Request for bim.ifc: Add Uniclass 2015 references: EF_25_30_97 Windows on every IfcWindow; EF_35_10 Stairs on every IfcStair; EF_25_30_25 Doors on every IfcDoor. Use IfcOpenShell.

First a look at what the model holds.

```python
import ifcopenshell

model = ifcopenshell.open("bim.ifc")
print(model.schema)
print("classifications:", [c.Name for c in model.by_type("IfcClassification")])
for ifc_class in ("IfcDoor", "IfcRoof", "IfcStair", "IfcWall", "IfcWindow"):
    print(ifc_class, len(model.by_type(ifc_class)))
```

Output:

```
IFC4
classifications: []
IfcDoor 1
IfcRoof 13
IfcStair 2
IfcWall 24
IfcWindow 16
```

```python
import ifcopenshell
import ifcopenshell.api.classification

model = ifcopenshell.open("bim.ifc")

system = ifcopenshell.api.classification.add_classification(model, classification="Uniclass 2015")

codes = {
    "IfcWindow": ("EF_25_30_97", "Windows"),
    "IfcStair": ("EF_35_10", "Stairs"),
    "IfcDoor": ("EF_25_30_25", "Doors"),
}
for ifc_class, (code, name) in codes.items():
    products = model.by_type(ifc_class)
    ifcopenshell.api.classification.add_reference(
        model, products=products, classification=system, identification=code, name=name
    )
    print(code, len(products))

model.write("bim_updated.ifc")
```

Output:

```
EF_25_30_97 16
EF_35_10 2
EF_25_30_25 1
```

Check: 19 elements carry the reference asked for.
